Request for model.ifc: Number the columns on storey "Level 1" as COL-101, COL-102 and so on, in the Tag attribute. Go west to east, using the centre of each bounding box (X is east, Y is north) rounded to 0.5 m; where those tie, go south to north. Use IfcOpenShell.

First a look at what the model holds.

```python
import ifcopenshell
import ifcopenshell.util.element
import ifcopenshell.util.placement

model = ifcopenshell.open("model.ifc")
print(model.schema)
storey = next(s for s in model.by_type("IfcBuildingStorey") if s.Name == "Level 1")
columns = [e for e in ifcopenshell.util.element.get_decomposition(storey) if e.is_a("IfcColumn")]
for e in sorted(columns, key=lambda e: e.id()):
    origin = ifcopenshell.util.placement.get_local_placement(e.ObjectPlacement)[:3, 3]
    print(e.id(), e.Tag, e.Name, origin.round(2) + 0.0, sep=" | ")
```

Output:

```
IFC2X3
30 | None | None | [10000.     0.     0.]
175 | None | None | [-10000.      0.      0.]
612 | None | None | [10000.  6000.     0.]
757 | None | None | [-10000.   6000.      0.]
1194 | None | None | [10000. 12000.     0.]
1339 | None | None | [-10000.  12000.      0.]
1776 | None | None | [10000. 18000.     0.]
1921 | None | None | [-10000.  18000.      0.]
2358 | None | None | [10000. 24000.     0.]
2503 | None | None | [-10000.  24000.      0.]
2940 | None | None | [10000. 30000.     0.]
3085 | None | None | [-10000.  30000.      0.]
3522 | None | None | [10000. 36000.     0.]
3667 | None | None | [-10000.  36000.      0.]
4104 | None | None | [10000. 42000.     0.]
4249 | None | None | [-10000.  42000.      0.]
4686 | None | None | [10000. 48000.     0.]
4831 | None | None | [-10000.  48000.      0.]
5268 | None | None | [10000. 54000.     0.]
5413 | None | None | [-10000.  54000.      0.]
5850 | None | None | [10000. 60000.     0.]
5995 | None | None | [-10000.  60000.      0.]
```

```python
import ifcopenshell
import ifcopenshell.geom
import ifcopenshell.util.element
import ifcopenshell.util.shape

model = ifcopenshell.open("model.ifc")
settings = ifcopenshell.geom.settings()
settings.set("use-world-coords", True)


def centre(element):
    shape = ifcopenshell.geom.create_shape(settings, element)
    return ifcopenshell.util.shape.get_bbox_centroid(shape.geometry)


storey = next(s for s in model.by_type("IfcBuildingStorey") if s.Name == "Level 1")
columns = [e for e in ifcopenshell.util.element.get_decomposition(storey) if e.is_a("IfcColumn")]

# Insertion points can sit at a corner or the storey origin, so sort by the geometry (in metres).
centres = {e: centre(e) for e in columns}
columns.sort(key=lambda e: (round(centres[e][0] / 0.5), centres[e][1]))

for i, e in enumerate(columns, start=1):
    number = f"COL-1{i:02d}"
    e.Tag = number
    print(e.id(), number)

model.write("model_v2.ifc")
```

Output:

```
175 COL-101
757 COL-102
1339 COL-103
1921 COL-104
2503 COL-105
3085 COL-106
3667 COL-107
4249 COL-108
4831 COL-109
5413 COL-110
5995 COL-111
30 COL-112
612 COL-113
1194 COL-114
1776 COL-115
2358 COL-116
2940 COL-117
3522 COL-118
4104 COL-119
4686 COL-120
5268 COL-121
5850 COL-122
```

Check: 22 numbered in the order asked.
